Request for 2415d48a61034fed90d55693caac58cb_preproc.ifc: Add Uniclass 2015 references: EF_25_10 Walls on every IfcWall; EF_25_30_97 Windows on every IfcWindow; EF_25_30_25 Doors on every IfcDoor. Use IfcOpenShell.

First a look at what the model holds.

```python
import ifcopenshell

model = ifcopenshell.open("2415d48a61034fed90d55693caac58cb_preproc.ifc")
print(model.schema)
print("classifications:", [c.Name for c in model.by_type("IfcClassification")])
for ifc_class in ("IfcDoor", "IfcRoof", "IfcStair", "IfcWall", "IfcWindow"):
    print(ifc_class, len(model.by_type(ifc_class)))
```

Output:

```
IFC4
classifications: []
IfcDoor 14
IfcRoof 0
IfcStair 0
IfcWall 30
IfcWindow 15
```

```python
import ifcopenshell
import ifcopenshell.api.classification

model = ifcopenshell.open("2415d48a61034fed90d55693caac58cb_preproc.ifc")

system = ifcopenshell.api.classification.add_classification(model, classification="Uniclass 2015")

codes = {
    "IfcWall": ("EF_25_10", "Walls"),
    "IfcWindow": ("EF_25_30_97", "Windows"),
    "IfcDoor": ("EF_25_30_25", "Doors"),
}
for ifc_class, (code, name) in codes.items():
    products = model.by_type(ifc_class)
    ifcopenshell.api.classification.add_reference(
        model, products=products, classification=system, identification=code, name=name
    )
    print(code, len(products))

model.write("2415d48a61034fed90d55693caac58cb_preproc_rev.ifc")
```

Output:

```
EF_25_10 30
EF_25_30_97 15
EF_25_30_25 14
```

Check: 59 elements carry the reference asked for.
